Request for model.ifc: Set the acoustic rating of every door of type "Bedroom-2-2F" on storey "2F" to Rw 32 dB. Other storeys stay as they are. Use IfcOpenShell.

First a look at what the model holds.

```python
import ifcopenshell
import ifcopenshell.util.element

model = ifcopenshell.open("model.ifc")
print(model.schema)
storey = next(s for s in model.by_type("IfcBuildingStorey") if s.Name == "2F")
doors = [e for e in ifcopenshell.util.element.get_decomposition(storey) if e.is_a("IfcDoor")]
seen = {}
for e in doors:
    element_type = ifcopenshell.util.element.get_type(e)
    key = (element_type.Name if element_type != e and element_type else None, ifcopenshell.util.element.get_pset(e, "Pset_DoorCommon", "AcousticRating"))
    seen[key] = seen.get(key, 0) + 1
for (name, value), count in sorted(seen.items(), key=str):
    print(count, "x", name, "|", value)
```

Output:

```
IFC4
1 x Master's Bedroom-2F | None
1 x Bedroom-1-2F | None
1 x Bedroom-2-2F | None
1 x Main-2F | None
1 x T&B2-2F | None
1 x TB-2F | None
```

```python
import ifcopenshell
import ifcopenshell.api.pset
import ifcopenshell.util.element

model = ifcopenshell.open("model.ifc")

storey = next(s for s in model.by_type("IfcBuildingStorey") if s.Name == "2F")
doors = [e for e in ifcopenshell.util.element.get_decomposition(storey) if e.is_a("IfcDoor")]

count = 0
for e in doors:
    element_type = ifcopenshell.util.element.get_type(e)
    if element_type in (None, e) or element_type.Name != "Bedroom-2-2F":
        continue
    # add_pset returns the element's existing set when there is one.
    pset = ifcopenshell.api.pset.add_pset(model, product=e, name="Pset_DoorCommon")
    ifcopenshell.api.pset.edit_pset(model, pset=pset, properties={"AcousticRating": "Rw 32 dB"})
    count += 1

print(count, "doors updated")

model.write("model_updated.ifc")
```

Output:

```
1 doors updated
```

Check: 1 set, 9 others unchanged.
